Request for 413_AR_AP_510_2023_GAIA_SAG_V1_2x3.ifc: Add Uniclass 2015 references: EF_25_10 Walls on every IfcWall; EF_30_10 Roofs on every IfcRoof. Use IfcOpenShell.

First a look at what the model holds.

```python
import ifcopenshell

model = ifcopenshell.open("413_AR_AP_510_2023_GAIA_SAG_V1_2x3.ifc")
print(model.schema)
print("classifications:", [c.Name for c in model.by_type("IfcClassification")])
for ifc_class in ("IfcDoor", "IfcRoof", "IfcStair", "IfcWall", "IfcWindow"):
    print(ifc_class, len(model.by_type(ifc_class)))
```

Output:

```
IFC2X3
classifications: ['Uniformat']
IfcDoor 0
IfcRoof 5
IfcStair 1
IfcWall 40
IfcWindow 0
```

```python
import ifcopenshell
import ifcopenshell.api.classification

model = ifcopenshell.open("413_AR_AP_510_2023_GAIA_SAG_V1_2x3.ifc")

# IFC2X3 requires Source and Edition and has no link from the project to the system.
system = model.create_entity("IfcClassification", Source="NBS", Edition="2015", Name="Uniclass 2015")

codes = {
    "IfcWall": ("EF_25_10", "Walls"),
    "IfcRoof": ("EF_30_10", "Roofs"),
}
for ifc_class, (code, name) in codes.items():
    products = model.by_type(ifc_class)
    ifcopenshell.api.classification.add_reference(
        model, products=products, classification=system, identification=code, name=name
    )
    print(code, len(products))

model.write("413_AR_AP_510_2023_GAIA_SAG_V1_2x3_edited.ifc")
```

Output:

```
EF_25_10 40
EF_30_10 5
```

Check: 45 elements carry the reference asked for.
